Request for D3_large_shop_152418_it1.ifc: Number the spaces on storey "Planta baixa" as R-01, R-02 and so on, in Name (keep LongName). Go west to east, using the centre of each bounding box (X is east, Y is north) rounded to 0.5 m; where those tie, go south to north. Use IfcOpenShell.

First a look at what the model holds.

```python
import ifcopenshell
import ifcopenshell.util.element
import ifcopenshell.util.placement

model = ifcopenshell.open("D3_large_shop_152418_it1.ifc")
print(model.schema)
storey = next(s for s in model.by_type("IfcBuildingStorey") if s.Name == "Planta baixa")
spaces = [e for e in ifcopenshell.util.element.get_decomposition(storey) if e.is_a("IfcSpace")]
for e in sorted(spaces, key=lambda e: e.id()):
    origin = ifcopenshell.util.placement.get_local_placement(e.ObjectPlacement)[:3, 3]
    print(e.id(), e.Name, e.LongName, origin.round(2) + 0.0, sep=" | ")
```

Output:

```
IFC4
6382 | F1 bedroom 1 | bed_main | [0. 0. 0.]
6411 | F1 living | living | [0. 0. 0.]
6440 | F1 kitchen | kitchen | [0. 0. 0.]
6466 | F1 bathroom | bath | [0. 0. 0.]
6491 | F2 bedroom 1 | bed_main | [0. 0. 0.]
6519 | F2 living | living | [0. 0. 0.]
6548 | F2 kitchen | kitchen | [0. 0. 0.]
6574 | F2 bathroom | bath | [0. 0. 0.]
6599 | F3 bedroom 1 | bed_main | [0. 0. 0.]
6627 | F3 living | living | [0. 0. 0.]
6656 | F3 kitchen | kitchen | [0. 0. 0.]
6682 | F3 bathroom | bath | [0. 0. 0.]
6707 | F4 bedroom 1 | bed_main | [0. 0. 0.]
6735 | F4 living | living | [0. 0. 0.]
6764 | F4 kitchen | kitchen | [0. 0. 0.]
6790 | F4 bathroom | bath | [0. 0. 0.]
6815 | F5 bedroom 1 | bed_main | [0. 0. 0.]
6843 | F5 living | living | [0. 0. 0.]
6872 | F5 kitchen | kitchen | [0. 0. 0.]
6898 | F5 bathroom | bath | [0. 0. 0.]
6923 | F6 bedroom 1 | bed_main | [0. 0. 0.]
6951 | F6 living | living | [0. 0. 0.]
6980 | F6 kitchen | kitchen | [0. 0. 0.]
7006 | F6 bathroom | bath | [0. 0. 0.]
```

```python
import ifcopenshell
import ifcopenshell.geom
import ifcopenshell.util.element
import ifcopenshell.util.shape

model = ifcopenshell.open("D3_large_shop_152418_it1.ifc")
settings = ifcopenshell.geom.settings()
settings.set("use-world-coords", True)


def centre(element):
    shape = ifcopenshell.geom.create_shape(settings, element)
    return ifcopenshell.util.shape.get_bbox_centroid(shape.geometry)


storey = next(s for s in model.by_type("IfcBuildingStorey") if s.Name == "Planta baixa")
spaces = [e for e in ifcopenshell.util.element.get_decomposition(storey) if e.is_a("IfcSpace")]

# Insertion points can sit at a corner or the storey origin, so sort by the geometry (in metres).
centres = {e: centre(e) for e in spaces}
spaces.sort(key=lambda e: (round(centres[e][0] / 0.5), centres[e][1]))

for i, e in enumerate(spaces, start=1):
    number = f"R-{i:02d}"
    e.Name = number
    print(e.id(), number)

model.write("D3_large_shop_152418_it1_rev.ifc")
```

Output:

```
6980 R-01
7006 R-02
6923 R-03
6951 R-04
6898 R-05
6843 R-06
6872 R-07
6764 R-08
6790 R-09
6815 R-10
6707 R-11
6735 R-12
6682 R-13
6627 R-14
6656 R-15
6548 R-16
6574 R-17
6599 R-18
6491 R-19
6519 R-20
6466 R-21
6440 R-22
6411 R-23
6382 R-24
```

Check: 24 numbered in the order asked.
